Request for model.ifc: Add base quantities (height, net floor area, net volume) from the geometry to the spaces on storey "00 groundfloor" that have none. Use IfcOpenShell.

First a look at what the model holds.

```python
import ifcopenshell
import ifcopenshell.util.element
import ifcopenshell.util.unit

model = ifcopenshell.open("model.ifc")
print(model.schema)
for unit_type in ("LENGTHUNIT", "AREAUNIT", "VOLUMEUNIT"):
    print(unit_type, ifcopenshell.util.unit.calculate_unit_scale(model, unit_type))
storey = next(s for s in model.by_type("IfcBuildingStorey") if s.Name == "00 groundfloor")
spaces = [e for e in ifcopenshell.util.element.get_decomposition(storey) if e.is_a("IfcSpace")]
for e in sorted(spaces, key=lambda e: e.id()):
    print(e.id(), e.is_a(), e.Name, list(ifcopenshell.util.element.get_psets(e, qtos_only=True)), sep=" | ")
```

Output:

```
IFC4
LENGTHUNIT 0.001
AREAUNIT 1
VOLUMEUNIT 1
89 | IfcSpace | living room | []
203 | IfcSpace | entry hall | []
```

```python
import ifcopenshell
import ifcopenshell.api.pset
import ifcopenshell.geom
import ifcopenshell.util.element
import ifcopenshell.util.shape
import ifcopenshell.util.unit

model = ifcopenshell.open("model.ifc")
unit_scale = ifcopenshell.util.unit.calculate_unit_scale(model)
area_scale = ifcopenshell.util.unit.calculate_unit_scale(model, "AREAUNIT")
volume_scale = ifcopenshell.util.unit.calculate_unit_scale(model, "VOLUMEUNIT")
settings = ifcopenshell.geom.settings()

storey = next(s for s in model.by_type("IfcBuildingStorey") if s.Name == "00 groundfloor")
spaces = [e for e in ifcopenshell.util.element.get_decomposition(storey) if e.is_a("IfcSpace")]

for e in sorted(spaces, key=lambda e: e.id()):
    if ifcopenshell.util.element.get_psets(e, qtos_only=True, should_inherit=False):
        continue
    # Geometry comes back in metres, in the element's own axes.
    shape = ifcopenshell.geom.create_shape(settings, e)
    values = {
        "Height": ifcopenshell.util.shape.get_z(shape.geometry) / unit_scale,
        "NetFloorArea": ifcopenshell.util.shape.get_footprint_area(shape.geometry) / area_scale,
        "NetVolume": ifcopenshell.util.shape.get_volume(shape.geometry) / volume_scale,
    }
    qto = ifcopenshell.api.pset.add_qto(model, product=e, name="Qto_SpaceBaseQuantities")
    ifcopenshell.api.pset.edit_qto(model, qto=qto, properties=values)
    print(e.id(), {k: round(v, 3) for k, v in values.items()})

model.write("model_updated.ifc")
```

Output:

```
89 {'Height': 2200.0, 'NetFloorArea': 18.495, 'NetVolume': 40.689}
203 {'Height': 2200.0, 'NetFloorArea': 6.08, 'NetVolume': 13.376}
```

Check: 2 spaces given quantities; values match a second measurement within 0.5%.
